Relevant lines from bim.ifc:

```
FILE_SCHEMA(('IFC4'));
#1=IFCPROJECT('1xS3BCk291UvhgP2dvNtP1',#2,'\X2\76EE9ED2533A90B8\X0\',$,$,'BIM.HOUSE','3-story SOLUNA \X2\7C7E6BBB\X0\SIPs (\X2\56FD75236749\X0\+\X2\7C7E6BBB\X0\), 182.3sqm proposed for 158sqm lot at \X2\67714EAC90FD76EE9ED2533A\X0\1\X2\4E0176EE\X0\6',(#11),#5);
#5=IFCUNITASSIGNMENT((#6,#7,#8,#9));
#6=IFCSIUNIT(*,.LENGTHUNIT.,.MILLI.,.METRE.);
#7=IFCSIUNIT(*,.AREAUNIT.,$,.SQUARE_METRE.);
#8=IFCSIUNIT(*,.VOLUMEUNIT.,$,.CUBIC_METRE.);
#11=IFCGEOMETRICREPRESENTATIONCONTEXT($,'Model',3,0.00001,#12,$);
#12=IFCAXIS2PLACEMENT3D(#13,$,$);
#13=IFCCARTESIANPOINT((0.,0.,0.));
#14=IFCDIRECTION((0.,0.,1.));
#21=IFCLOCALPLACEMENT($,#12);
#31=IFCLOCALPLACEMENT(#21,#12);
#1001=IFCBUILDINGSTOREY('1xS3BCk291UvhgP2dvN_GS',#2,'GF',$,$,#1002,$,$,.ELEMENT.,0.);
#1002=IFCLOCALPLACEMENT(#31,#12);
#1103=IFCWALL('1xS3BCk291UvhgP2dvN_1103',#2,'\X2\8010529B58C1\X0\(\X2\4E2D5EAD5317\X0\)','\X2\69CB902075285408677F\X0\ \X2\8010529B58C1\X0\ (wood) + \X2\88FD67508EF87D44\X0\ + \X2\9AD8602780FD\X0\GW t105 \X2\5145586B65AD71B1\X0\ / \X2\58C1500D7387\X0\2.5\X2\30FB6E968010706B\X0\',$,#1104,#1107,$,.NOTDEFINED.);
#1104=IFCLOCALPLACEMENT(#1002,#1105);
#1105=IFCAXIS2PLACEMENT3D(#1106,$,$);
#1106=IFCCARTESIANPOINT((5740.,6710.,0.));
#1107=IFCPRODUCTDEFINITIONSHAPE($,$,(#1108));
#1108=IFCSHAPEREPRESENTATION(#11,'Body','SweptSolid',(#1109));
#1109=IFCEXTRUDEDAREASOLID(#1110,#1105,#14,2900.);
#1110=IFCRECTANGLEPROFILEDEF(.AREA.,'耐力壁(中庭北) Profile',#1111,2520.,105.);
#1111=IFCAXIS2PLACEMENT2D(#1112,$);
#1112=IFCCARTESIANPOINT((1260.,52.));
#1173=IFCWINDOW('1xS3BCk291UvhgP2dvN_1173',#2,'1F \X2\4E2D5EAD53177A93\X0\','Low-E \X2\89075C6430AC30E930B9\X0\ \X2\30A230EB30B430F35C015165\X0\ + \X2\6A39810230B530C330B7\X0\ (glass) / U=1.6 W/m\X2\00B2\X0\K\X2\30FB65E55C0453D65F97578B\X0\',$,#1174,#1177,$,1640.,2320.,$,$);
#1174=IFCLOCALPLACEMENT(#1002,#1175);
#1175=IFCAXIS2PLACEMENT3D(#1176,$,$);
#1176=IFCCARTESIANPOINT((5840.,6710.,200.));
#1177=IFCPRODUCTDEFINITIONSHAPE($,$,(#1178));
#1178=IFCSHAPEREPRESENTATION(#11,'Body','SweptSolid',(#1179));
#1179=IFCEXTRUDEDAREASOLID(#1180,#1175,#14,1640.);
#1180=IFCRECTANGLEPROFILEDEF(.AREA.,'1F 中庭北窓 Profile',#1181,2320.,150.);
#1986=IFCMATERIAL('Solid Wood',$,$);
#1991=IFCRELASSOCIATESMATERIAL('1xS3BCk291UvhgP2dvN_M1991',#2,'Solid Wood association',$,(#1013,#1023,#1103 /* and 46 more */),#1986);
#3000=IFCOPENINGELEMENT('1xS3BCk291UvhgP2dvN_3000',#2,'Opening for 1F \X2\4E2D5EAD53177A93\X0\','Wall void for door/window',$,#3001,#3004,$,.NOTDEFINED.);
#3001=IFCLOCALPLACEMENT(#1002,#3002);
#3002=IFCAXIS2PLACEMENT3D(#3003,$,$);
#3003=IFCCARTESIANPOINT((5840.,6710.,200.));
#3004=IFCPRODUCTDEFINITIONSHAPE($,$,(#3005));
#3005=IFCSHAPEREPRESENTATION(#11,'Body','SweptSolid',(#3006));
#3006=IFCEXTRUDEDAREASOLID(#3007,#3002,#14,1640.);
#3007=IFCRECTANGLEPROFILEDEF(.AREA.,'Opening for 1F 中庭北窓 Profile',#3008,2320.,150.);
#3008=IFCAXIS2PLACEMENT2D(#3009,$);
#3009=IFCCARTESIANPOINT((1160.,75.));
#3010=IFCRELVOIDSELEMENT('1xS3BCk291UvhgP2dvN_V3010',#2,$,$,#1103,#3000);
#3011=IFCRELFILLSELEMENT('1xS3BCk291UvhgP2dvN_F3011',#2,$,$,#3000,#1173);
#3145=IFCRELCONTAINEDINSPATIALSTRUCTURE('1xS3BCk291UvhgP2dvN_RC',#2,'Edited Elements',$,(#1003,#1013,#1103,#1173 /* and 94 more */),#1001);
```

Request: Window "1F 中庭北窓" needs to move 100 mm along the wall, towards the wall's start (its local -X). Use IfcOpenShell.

```python
import ifcopenshell
import ifcopenshell.api.geometry
import ifcopenshell.util.placement
import ifcopenshell.util.unit

model = ifcopenshell.open("bim.ifc")
unit_scale = ifcopenshell.util.unit.calculate_unit_scale(model)

window = model.by_id(1173)
opening = window.FillsVoids[0].RelatingOpeningElement
wall = opening.VoidsElements[0].RelatingBuildingElement

wall_matrix = ifcopenshell.util.placement.get_local_placement(wall.ObjectPlacement)
shift = wall_matrix[:3, 0] * -0.1 / unit_scale
before = ifcopenshell.util.placement.get_local_placement(window.ObjectPlacement)[:3, 3].copy()

# The window is not placed relative to its opening, so move both.
for product in (opening, window):
    matrix = ifcopenshell.util.placement.get_local_placement(product.ObjectPlacement)
    matrix[:3, 3] += shift
    ifcopenshell.api.geometry.edit_object_placement(model, product=product, matrix=matrix, is_si=False)

after = ifcopenshell.util.placement.get_local_placement(window.ObjectPlacement)[:3, 3]
print("window moved by", (after - before).round(3) + 0.0)

model.write("bim_updated.ifc")
```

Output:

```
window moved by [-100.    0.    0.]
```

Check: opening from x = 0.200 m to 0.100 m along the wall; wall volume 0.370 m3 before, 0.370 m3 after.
